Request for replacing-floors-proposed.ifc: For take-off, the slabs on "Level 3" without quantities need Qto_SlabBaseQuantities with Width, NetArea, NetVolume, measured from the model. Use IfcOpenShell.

First a look at what the model holds.

```python
import ifcopenshell
import ifcopenshell.util.element
import ifcopenshell.util.unit

model = ifcopenshell.open("replacing-floors-proposed.ifc")
print(model.schema)
for unit_type in ("LENGTHUNIT", "AREAUNIT", "VOLUMEUNIT"):
    print(unit_type, ifcopenshell.util.unit.calculate_unit_scale(model, unit_type))
storey = next(s for s in model.by_type("IfcBuildingStorey") if s.Name == "Level 3")
slabs = [e for e in ifcopenshell.util.element.get_decomposition(storey) if e.is_a("IfcSlab")]
for e in sorted(slabs, key=lambda e: e.id()):
    print(e.id(), e.is_a(), e.Name, list(ifcopenshell.util.element.get_psets(e, qtos_only=True)), sep=" | ")
```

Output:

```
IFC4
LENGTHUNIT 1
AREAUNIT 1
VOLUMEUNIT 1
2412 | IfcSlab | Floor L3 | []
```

```python
import ifcopenshell
import ifcopenshell.api.pset
import ifcopenshell.geom
import ifcopenshell.util.element
import ifcopenshell.util.shape
import ifcopenshell.util.unit

model = ifcopenshell.open("replacing-floors-proposed.ifc")
unit_scale = ifcopenshell.util.unit.calculate_unit_scale(model)
area_scale = ifcopenshell.util.unit.calculate_unit_scale(model, "AREAUNIT")
volume_scale = ifcopenshell.util.unit.calculate_unit_scale(model, "VOLUMEUNIT")
settings = ifcopenshell.geom.settings()

storey = next(s for s in model.by_type("IfcBuildingStorey") if s.Name == "Level 3")
slabs = [e for e in ifcopenshell.util.element.get_decomposition(storey) if e.is_a("IfcSlab")]

for e in sorted(slabs, key=lambda e: e.id()):
    if ifcopenshell.util.element.get_psets(e, qtos_only=True, should_inherit=False):
        continue
    # Geometry comes back in metres, in the element's own axes.
    shape = ifcopenshell.geom.create_shape(settings, e)
    values = {
        "Width": ifcopenshell.util.shape.get_z(shape.geometry) / unit_scale,
        "NetArea": ifcopenshell.util.shape.get_footprint_area(shape.geometry) / area_scale,
        "NetVolume": ifcopenshell.util.shape.get_volume(shape.geometry) / volume_scale,
    }
    qto = ifcopenshell.api.pset.add_qto(model, product=e, name="Qto_SlabBaseQuantities")
    ifcopenshell.api.pset.edit_qto(model, qto=qto, properties=values)
    print(e.id(), {k: round(v, 3) for k, v in values.items()})

model.write("replacing-floors-proposed_updated.ifc")
```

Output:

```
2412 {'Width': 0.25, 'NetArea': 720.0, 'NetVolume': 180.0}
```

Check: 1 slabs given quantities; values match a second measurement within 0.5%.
